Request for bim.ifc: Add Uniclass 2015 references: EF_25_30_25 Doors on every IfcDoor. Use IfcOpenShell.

First a look at what the model holds.

```python
import ifcopenshell

model = ifcopenshell.open("bim.ifc")
print(model.schema)
print("classifications:", [c.Name for c in model.by_type("IfcClassification")])
for ifc_class in ("IfcDoor", "IfcRoof", "IfcStair", "IfcWall", "IfcWindow"):
    print(ifc_class, len(model.by_type(ifc_class)))
```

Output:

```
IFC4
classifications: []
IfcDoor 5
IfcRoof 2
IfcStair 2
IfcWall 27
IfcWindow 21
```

```python
import ifcopenshell
import ifcopenshell.api.classification

model = ifcopenshell.open("bim.ifc")

system = ifcopenshell.api.classification.add_classification(model, classification="Uniclass 2015")

codes = {
    "IfcDoor": ("EF_25_30_25", "Doors"),
}
for ifc_class, (code, name) in codes.items():
    products = model.by_type(ifc_class)
    ifcopenshell.api.classification.add_reference(
        model, products=products, classification=system, identification=code, name=name
    )
    print(code, len(products))

model.write("bim_rev.ifc")
```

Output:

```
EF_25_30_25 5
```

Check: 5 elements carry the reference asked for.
